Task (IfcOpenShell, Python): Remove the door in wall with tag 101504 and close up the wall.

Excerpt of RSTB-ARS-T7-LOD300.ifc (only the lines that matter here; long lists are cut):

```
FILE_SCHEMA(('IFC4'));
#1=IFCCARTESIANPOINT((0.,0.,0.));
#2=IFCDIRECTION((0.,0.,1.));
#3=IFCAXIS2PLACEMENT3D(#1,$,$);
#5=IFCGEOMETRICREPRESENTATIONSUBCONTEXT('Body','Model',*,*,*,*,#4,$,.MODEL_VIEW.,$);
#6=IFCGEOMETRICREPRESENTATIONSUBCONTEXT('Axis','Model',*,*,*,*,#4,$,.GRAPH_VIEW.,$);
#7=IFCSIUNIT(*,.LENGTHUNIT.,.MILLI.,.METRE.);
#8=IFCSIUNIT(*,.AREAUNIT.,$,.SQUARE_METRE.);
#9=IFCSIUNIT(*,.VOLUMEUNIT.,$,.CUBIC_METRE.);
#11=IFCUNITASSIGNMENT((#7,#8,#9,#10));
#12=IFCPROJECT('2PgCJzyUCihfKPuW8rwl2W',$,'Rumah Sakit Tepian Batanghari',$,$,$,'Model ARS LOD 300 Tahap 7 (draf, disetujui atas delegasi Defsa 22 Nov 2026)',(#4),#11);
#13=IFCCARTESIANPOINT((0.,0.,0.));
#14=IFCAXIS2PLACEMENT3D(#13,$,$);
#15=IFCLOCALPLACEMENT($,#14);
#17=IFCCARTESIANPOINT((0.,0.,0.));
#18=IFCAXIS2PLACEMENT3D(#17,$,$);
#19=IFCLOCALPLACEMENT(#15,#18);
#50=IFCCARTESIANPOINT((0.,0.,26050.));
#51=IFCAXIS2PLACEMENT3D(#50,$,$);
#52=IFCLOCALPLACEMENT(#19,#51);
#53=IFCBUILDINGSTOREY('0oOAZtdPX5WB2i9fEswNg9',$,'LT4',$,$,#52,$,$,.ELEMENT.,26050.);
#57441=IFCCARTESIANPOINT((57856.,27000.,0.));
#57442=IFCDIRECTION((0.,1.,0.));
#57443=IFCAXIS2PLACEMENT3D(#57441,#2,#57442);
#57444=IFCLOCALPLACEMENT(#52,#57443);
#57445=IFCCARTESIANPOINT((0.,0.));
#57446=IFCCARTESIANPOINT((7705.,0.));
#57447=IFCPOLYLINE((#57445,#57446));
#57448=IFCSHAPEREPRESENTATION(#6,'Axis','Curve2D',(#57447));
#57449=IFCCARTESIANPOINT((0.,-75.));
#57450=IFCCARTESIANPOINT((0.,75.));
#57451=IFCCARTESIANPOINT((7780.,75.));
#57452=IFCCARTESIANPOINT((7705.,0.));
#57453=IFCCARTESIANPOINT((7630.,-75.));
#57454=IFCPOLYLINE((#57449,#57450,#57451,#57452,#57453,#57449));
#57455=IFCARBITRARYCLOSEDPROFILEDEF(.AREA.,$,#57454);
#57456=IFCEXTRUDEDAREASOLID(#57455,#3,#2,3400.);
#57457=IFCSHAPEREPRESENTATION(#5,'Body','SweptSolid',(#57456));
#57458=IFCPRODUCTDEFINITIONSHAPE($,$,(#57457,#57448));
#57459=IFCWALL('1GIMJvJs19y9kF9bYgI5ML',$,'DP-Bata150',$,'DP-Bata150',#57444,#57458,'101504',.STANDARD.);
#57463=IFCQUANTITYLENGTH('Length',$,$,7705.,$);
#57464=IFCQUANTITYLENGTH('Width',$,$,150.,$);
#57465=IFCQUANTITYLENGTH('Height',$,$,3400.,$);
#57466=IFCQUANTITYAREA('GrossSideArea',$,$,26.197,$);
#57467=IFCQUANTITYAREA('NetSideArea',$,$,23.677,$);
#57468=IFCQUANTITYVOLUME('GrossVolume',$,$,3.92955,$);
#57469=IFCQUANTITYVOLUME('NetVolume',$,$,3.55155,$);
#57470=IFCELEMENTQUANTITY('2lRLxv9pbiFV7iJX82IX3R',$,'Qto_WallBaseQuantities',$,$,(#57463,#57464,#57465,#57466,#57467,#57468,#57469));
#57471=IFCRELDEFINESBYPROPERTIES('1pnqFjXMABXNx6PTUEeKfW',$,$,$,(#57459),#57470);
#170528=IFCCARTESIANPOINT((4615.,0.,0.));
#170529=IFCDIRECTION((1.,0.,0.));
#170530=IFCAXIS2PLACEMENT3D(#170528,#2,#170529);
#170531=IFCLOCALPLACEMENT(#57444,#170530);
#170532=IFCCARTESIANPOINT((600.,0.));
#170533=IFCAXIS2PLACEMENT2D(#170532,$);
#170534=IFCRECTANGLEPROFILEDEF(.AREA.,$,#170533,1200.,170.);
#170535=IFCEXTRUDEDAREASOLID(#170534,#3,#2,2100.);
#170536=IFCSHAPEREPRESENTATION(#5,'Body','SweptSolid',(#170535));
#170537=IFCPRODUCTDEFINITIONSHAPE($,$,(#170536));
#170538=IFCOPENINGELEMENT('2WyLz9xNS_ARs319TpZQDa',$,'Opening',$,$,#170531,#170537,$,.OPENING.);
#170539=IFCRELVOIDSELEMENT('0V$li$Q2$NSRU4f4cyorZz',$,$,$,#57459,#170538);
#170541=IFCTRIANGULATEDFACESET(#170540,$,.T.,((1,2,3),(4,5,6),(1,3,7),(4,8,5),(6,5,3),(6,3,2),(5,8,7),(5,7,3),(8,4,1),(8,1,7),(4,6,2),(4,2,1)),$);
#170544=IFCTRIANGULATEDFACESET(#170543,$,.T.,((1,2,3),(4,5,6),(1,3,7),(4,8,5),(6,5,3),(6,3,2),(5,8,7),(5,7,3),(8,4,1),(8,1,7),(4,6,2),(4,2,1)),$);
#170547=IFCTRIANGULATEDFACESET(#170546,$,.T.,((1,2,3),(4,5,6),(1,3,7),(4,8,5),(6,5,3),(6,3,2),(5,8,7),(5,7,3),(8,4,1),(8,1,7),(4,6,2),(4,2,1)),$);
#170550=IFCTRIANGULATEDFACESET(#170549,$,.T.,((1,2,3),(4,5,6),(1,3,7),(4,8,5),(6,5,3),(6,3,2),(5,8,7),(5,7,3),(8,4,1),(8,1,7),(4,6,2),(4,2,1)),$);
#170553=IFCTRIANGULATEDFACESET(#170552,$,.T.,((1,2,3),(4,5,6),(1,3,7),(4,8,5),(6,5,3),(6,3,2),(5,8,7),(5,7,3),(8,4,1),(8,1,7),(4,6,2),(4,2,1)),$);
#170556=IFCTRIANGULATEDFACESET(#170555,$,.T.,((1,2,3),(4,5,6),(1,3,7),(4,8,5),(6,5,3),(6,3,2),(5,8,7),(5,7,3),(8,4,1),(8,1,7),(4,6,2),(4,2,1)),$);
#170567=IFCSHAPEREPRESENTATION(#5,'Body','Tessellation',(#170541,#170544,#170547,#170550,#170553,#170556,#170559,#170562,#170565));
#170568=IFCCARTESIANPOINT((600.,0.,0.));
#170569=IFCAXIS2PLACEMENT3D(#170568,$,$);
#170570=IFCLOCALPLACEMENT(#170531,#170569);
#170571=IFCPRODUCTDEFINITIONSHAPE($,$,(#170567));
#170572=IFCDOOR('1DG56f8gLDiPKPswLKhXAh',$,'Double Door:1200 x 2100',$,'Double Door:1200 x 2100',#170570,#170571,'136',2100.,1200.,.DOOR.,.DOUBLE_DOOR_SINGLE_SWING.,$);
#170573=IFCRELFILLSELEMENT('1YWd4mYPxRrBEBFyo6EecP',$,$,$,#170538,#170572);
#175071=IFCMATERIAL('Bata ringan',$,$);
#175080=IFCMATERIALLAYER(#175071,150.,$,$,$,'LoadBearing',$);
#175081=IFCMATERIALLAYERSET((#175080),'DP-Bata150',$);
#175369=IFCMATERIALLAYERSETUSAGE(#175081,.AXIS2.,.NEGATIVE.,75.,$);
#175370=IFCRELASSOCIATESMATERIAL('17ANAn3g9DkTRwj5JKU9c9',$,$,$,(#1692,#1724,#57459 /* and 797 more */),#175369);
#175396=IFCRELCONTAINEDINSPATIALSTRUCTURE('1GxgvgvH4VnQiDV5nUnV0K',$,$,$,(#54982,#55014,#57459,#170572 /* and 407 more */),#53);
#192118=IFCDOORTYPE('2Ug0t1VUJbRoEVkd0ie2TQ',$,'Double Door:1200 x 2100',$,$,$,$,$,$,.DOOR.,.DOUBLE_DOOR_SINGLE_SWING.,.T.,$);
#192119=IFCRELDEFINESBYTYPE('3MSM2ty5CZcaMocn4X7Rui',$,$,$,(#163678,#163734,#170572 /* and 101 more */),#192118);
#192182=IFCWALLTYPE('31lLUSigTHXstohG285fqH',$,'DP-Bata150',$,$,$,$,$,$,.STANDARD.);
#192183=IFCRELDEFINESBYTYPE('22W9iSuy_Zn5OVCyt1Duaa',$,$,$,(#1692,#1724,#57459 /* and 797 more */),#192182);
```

```python
import ifcopenshell
import ifcopenshell.api.feature
import ifcopenshell.api.pset
import ifcopenshell.api.root
import ifcopenshell.geom
import ifcopenshell.util.element
import ifcopenshell.util.shape
import ifcopenshell.util.unit

model = ifcopenshell.open("RSTB-ARS-T7-LOD300.ifc")
area_scale = ifcopenshell.util.unit.calculate_unit_scale(model, "AREAUNIT")
volume_scale = ifcopenshell.util.unit.calculate_unit_scale(model, "VOLUMEUNIT")
settings = ifcopenshell.geom.settings()


def volume(element):
    """Net volume in cubic metres, openings subtracted."""
    shape = ifcopenshell.geom.create_shape(settings, element)
    return ifcopenshell.util.shape.get_volume(shape.geometry)


door = model.by_guid("1DG56f8gLDiPKPswLKhXAh")
opening = door.FillsVoids[0].RelatingOpeningElement
wall = opening.VoidsElements[0].RelatingBuildingElement
before = volume(wall)

ifcopenshell.api.root.remove_product(model, product=door)
ifcopenshell.api.feature.remove_feature(model, feature=opening)

after = volume(wall)
thickness = 0.15  # wall thickness in metres

# Update the wall's stored quantities.
qto = model.by_id(ifcopenshell.util.element.get_pset(wall, "Qto_WallBaseQuantities", should_inherit=False)["id"])
ifcopenshell.api.pset.edit_qto(model, qto=qto, properties={
    "NetSideArea": after / thickness / area_scale,
    "NetVolume": after / volume_scale,
})

print(f"wall volume {before:.3f} -> {after:.3f} m3")

model.write("RSTB-ARS-T7-LOD300_updated.ifc")
```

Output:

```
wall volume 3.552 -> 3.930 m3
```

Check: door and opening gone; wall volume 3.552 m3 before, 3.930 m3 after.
